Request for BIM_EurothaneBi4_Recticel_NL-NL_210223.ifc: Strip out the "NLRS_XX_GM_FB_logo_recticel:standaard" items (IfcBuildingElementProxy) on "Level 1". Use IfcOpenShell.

First a look at what the model holds.

```python
import ifcopenshell
import ifcopenshell.util.element

model = ifcopenshell.open("BIM_EurothaneBi4_Recticel_NL-NL_210223.ifc")
print(model.schema)
storey = next(s for s in model.by_type("IfcBuildingStorey") if s.Name == "Level 1")
proxies = [e for e in ifcopenshell.util.element.get_decomposition(storey) if e.is_a("IfcBuildingElementProxy")]
seen = {}
for e in proxies:
    element_type = ifcopenshell.util.element.get_type(e)
    name = element_type.Name if element_type not in (None, e) else None
    seen[name] = seen.get(name, 0) + 1
for name, count in sorted(seen.items(), key=str):
    print(count, "x", name)
```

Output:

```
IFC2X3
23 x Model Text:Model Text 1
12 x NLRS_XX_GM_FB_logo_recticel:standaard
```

```python
import ifcopenshell
import ifcopenshell.api.root
import ifcopenshell.util.element

model = ifcopenshell.open("BIM_EurothaneBi4_Recticel_NL-NL_210223.ifc")

storey = next(s for s in model.by_type("IfcBuildingStorey") if s.Name == "Level 1")
proxies = [e for e in ifcopenshell.util.element.get_decomposition(storey) if e.is_a("IfcBuildingElementProxy")]
targets = [e for e in proxies if (t := ifcopenshell.util.element.get_type(e)) not in (None, e) and t.Name == "NLRS_XX_GM_FB_logo_recticel:standaard"]

for e in targets:
    ifcopenshell.api.root.remove_product(model, product=e)
print(len(targets), "removed")

model.write("BIM_EurothaneBi4_Recticel_NL-NL_210223_rev.ifc")
```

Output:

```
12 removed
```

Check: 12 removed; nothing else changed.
